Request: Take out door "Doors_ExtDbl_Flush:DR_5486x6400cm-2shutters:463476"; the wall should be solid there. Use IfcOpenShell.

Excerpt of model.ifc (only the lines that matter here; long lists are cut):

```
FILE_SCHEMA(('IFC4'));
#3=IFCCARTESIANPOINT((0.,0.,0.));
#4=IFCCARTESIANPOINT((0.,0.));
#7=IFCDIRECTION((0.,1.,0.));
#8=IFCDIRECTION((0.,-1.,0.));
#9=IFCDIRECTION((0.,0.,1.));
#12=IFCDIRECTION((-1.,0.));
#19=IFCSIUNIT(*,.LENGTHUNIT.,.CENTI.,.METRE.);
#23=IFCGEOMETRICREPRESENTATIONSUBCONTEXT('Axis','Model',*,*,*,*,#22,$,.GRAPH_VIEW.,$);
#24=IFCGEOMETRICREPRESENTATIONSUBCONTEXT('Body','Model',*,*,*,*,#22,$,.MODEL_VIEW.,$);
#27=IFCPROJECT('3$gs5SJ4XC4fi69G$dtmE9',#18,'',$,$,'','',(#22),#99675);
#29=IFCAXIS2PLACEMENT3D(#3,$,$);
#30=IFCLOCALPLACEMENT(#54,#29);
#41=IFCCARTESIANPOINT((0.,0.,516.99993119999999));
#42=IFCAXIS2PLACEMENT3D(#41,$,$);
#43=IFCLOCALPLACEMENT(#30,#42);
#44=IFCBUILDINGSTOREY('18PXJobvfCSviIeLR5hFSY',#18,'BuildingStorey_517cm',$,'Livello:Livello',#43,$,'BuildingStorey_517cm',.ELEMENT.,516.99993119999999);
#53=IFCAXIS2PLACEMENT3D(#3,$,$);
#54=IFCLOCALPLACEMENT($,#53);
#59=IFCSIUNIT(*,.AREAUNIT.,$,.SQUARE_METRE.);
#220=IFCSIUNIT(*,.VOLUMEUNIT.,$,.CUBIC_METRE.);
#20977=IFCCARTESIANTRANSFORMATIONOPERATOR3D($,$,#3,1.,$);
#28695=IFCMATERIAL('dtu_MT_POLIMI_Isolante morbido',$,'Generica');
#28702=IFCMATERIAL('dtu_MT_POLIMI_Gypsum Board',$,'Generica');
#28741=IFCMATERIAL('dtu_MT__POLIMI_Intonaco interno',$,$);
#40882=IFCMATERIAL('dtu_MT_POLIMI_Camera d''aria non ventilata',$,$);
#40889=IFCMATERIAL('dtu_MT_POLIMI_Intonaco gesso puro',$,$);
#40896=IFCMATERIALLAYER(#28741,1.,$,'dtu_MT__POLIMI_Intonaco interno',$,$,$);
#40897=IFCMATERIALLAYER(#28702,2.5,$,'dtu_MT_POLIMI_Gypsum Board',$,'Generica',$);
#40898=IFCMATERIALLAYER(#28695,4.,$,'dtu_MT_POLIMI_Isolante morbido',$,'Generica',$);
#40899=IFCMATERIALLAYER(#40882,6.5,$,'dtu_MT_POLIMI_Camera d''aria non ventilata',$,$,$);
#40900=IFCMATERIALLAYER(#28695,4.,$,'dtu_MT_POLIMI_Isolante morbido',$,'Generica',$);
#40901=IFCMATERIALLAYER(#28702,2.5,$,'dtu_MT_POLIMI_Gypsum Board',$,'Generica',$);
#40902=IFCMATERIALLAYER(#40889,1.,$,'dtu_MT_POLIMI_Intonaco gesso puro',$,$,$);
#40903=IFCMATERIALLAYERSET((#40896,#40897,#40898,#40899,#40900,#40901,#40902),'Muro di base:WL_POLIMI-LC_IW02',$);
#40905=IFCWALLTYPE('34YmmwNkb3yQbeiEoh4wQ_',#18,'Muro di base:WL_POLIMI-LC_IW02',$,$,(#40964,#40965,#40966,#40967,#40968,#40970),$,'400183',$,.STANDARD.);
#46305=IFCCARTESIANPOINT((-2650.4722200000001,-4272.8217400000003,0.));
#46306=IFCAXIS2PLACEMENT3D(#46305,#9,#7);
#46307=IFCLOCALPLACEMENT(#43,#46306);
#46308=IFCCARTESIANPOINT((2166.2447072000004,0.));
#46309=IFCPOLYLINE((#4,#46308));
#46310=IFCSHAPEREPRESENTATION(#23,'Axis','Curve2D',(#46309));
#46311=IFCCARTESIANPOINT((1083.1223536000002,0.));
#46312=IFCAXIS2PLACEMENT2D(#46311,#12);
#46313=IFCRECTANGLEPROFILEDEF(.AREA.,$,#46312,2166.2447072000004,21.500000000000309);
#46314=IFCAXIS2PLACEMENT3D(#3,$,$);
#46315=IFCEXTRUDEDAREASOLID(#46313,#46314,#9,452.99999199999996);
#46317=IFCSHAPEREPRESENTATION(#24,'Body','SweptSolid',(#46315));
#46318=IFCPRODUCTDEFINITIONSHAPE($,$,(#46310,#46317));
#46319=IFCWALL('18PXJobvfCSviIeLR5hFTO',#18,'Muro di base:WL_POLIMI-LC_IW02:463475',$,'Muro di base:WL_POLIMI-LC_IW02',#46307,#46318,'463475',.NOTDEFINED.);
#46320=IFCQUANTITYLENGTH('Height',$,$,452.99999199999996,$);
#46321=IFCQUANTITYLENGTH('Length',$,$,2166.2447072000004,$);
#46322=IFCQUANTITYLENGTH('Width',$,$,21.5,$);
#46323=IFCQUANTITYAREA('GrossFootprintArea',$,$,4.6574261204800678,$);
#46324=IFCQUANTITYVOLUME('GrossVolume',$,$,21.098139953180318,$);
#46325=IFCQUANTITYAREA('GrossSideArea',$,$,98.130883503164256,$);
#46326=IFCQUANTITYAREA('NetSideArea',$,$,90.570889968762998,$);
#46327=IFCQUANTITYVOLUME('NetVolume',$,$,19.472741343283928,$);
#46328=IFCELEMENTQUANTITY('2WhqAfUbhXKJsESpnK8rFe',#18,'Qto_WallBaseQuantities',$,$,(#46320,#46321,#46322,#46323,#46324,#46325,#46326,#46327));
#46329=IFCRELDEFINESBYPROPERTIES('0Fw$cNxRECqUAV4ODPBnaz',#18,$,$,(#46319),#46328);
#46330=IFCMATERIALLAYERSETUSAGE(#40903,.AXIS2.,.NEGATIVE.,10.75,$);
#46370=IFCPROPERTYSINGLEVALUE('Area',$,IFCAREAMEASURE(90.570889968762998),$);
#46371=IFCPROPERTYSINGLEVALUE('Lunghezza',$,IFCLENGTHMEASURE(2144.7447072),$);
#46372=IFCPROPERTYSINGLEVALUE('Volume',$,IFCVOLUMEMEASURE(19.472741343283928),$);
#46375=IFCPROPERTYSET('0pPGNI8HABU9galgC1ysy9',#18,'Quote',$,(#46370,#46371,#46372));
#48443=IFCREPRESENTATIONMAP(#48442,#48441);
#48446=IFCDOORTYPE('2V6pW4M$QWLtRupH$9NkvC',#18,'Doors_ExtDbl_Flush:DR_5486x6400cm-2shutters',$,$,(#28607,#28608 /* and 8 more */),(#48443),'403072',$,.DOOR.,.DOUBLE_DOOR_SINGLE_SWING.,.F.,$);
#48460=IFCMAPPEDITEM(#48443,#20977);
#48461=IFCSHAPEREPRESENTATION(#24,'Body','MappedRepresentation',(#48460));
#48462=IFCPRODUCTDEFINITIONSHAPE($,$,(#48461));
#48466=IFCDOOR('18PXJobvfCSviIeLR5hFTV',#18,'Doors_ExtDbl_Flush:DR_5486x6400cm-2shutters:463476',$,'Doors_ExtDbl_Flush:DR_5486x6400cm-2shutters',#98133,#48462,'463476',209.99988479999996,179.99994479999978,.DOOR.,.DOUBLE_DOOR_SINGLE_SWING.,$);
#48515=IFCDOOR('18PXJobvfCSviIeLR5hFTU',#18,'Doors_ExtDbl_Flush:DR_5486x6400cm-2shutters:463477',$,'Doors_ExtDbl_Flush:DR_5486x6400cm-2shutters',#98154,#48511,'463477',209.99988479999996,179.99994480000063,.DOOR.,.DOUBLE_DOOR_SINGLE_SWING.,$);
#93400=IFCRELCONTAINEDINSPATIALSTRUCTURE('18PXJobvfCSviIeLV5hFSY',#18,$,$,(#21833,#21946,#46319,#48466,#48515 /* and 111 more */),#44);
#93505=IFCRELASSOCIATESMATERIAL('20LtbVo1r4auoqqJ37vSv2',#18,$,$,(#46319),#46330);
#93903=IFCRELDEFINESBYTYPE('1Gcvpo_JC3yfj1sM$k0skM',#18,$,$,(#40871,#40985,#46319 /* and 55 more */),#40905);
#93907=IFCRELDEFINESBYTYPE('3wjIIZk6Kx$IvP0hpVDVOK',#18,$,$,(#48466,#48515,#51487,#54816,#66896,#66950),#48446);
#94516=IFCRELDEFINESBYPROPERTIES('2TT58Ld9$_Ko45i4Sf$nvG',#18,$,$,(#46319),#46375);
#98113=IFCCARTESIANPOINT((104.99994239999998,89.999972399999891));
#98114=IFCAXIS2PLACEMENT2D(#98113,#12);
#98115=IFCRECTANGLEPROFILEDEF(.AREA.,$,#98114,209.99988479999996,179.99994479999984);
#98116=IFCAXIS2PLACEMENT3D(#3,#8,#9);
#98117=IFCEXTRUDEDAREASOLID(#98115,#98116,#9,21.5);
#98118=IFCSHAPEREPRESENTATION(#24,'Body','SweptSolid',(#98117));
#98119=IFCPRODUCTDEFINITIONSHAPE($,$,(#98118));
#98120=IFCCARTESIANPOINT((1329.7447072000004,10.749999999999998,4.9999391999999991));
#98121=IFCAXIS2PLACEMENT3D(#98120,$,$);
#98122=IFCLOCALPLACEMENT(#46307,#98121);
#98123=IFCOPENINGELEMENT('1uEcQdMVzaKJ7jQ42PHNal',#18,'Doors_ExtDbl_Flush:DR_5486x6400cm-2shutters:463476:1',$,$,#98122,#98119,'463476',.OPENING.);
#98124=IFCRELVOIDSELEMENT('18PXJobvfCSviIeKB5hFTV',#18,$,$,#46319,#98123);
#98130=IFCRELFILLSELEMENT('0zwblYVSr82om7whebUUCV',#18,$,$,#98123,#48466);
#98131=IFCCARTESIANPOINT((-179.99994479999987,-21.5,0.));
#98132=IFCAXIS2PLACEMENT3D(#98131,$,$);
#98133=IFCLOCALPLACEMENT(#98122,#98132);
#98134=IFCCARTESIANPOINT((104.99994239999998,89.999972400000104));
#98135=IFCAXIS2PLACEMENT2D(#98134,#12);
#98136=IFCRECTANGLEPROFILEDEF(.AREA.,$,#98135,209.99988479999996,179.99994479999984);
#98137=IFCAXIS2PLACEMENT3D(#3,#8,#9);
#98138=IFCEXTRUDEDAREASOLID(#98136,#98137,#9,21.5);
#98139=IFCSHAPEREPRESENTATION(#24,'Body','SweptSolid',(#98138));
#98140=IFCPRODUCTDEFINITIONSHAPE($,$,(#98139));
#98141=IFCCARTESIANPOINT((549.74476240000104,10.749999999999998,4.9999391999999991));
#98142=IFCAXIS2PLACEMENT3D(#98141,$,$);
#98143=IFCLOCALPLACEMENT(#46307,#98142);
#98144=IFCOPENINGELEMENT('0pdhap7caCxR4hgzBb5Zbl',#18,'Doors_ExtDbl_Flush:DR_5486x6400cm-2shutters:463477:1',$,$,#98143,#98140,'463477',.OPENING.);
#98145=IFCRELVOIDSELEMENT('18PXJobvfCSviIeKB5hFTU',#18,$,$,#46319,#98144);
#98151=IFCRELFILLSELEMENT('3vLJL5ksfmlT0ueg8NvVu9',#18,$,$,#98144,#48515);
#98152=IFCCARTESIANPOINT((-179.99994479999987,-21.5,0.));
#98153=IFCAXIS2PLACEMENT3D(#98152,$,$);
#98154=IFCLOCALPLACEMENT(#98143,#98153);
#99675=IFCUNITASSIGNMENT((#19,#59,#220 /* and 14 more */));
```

```python
import ifcopenshell
import ifcopenshell.api.feature
import ifcopenshell.api.pset
import ifcopenshell.api.root
import ifcopenshell.geom
import ifcopenshell.util.element
import ifcopenshell.util.shape
import ifcopenshell.util.unit

model = ifcopenshell.open("model.ifc")
area_scale = ifcopenshell.util.unit.calculate_unit_scale(model, "AREAUNIT")
volume_scale = ifcopenshell.util.unit.calculate_unit_scale(model, "VOLUMEUNIT")
settings = ifcopenshell.geom.settings()


def volume(element):
    """Net volume in cubic metres, openings subtracted."""
    shape = ifcopenshell.geom.create_shape(settings, element)
    return ifcopenshell.util.shape.get_volume(shape.geometry)


door = model.by_guid("18PXJobvfCSviIeLR5hFTV")
opening = door.FillsVoids[0].RelatingOpeningElement
wall = opening.VoidsElements[0].RelatingBuildingElement
before = volume(wall)

ifcopenshell.api.root.remove_product(model, product=door)
ifcopenshell.api.feature.remove_feature(model, feature=opening)

after = volume(wall)
thickness = 0.215  # wall thickness in metres

# Update the wall's stored quantities.
qto = model.by_id(ifcopenshell.util.element.get_pset(wall, "Qto_WallBaseQuantities", should_inherit=False)["id"])
ifcopenshell.api.pset.edit_qto(model, qto=qto, properties={
    "NetSideArea": after / thickness / area_scale,
    "NetVolume": after / volume_scale,
})
pset = model.by_id(ifcopenshell.util.element.get_pset(wall, "Quote", should_inherit=False)["id"])
ifcopenshell.api.pset.edit_pset(model, pset=pset, properties={
    "Area": model.create_entity("IfcAreaMeasure", after / thickness / area_scale),
    "Volume": model.create_entity("IfcVolumeMeasure", after / volume_scale),
})

print(f"wall volume {before:.3f} -> {after:.3f} m3")

model.write("model_updated.ifc")
```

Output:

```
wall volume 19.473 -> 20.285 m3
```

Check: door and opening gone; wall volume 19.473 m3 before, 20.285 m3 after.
